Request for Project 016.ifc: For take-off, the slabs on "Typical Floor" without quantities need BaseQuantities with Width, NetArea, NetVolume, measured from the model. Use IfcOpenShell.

First a look at what the model holds.

```python
import ifcopenshell
import ifcopenshell.util.element
import ifcopenshell.util.unit

model = ifcopenshell.open("Project 016.ifc")
print(model.schema)
for unit_type in ("LENGTHUNIT", "AREAUNIT", "VOLUMEUNIT"):
    print(unit_type, ifcopenshell.util.unit.calculate_unit_scale(model, unit_type))
storey = next(s for s in model.by_type("IfcBuildingStorey") if s.Name == "Typical Floor")
slabs = [e for e in ifcopenshell.util.element.get_decomposition(storey) if e.is_a("IfcSlab")]
for e in sorted(slabs, key=lambda e: e.id()):
    print(e.id(), e.is_a(), e.Name, list(ifcopenshell.util.element.get_psets(e, qtos_only=True)), sep=" | ")
```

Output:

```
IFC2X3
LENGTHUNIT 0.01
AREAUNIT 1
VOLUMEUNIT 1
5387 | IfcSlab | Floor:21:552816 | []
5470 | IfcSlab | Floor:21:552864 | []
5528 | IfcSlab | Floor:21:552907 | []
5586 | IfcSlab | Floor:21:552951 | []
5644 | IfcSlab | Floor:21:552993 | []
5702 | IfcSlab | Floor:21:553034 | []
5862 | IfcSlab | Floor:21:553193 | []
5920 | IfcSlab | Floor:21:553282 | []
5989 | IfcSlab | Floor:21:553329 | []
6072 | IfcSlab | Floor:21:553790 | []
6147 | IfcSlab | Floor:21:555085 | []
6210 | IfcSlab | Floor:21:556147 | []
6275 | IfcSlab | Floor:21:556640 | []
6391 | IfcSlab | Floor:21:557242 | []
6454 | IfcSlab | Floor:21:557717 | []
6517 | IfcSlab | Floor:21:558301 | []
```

```python
import ifcopenshell
import ifcopenshell.api.pset
import ifcopenshell.geom
import ifcopenshell.util.element
import ifcopenshell.util.shape
import ifcopenshell.util.unit

model = ifcopenshell.open("Project 016.ifc")
unit_scale = ifcopenshell.util.unit.calculate_unit_scale(model)
area_scale = ifcopenshell.util.unit.calculate_unit_scale(model, "AREAUNIT")
volume_scale = ifcopenshell.util.unit.calculate_unit_scale(model, "VOLUMEUNIT")
settings = ifcopenshell.geom.settings()

storey = next(s for s in model.by_type("IfcBuildingStorey") if s.Name == "Typical Floor")
slabs = [e for e in ifcopenshell.util.element.get_decomposition(storey) if e.is_a("IfcSlab")]

for e in sorted(slabs, key=lambda e: e.id()):
    if ifcopenshell.util.element.get_psets(e, qtos_only=True, should_inherit=False):
        continue
    # Geometry comes back in metres, in the element's own axes.
    shape = ifcopenshell.geom.create_shape(settings, e)
    values = {
        "Width": ifcopenshell.util.shape.get_z(shape.geometry) / unit_scale,
        "NetArea": ifcopenshell.util.shape.get_footprint_area(shape.geometry) / area_scale,
        "NetVolume": ifcopenshell.util.shape.get_volume(shape.geometry) / volume_scale,
    }
    qto = ifcopenshell.api.pset.add_qto(model, product=e, name="BaseQuantities")
    ifcopenshell.api.pset.edit_qto(model, qto=qto, properties=values)
    print(e.id(), {k: round(v, 3) for k, v in values.items()})

model.write("Project 016_edited.ifc")
```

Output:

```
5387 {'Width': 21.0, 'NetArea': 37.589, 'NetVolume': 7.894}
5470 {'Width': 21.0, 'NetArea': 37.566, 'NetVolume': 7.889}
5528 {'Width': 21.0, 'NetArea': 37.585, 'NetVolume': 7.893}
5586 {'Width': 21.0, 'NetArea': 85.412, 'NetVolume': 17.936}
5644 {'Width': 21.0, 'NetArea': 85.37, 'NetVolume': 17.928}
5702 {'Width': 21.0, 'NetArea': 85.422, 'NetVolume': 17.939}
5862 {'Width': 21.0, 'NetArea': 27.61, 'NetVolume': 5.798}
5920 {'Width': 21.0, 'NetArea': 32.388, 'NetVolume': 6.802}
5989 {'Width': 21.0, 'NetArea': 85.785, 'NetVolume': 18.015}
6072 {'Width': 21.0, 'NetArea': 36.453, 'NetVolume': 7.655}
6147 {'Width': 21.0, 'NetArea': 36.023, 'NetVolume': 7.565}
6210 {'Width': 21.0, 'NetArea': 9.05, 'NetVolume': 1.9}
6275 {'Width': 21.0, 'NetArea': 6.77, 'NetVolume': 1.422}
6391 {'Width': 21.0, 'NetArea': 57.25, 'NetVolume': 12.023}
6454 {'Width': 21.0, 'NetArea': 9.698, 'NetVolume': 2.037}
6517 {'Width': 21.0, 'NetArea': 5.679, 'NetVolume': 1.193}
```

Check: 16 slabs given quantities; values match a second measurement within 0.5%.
